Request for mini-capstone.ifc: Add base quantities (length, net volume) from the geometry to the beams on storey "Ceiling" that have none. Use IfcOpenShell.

First a look at what the model holds.

```python
import ifcopenshell
import ifcopenshell.util.element
import ifcopenshell.util.unit

model = ifcopenshell.open("mini-capstone.ifc")
print(model.schema)
for unit_type in ("LENGTHUNIT", "AREAUNIT", "VOLUMEUNIT"):
    print(unit_type, ifcopenshell.util.unit.calculate_unit_scale(model, unit_type))
storey = next(s for s in model.by_type("IfcBuildingStorey") if s.Name == "Ceiling")
beams = [e for e in ifcopenshell.util.element.get_decomposition(storey) if e.is_a("IfcBeam")]
for e in sorted(beams, key=lambda e: e.id()):
    print(e.id(), e.is_a(), e.Name, list(ifcopenshell.util.element.get_psets(e, qtos_only=True)), sep=" | ")
```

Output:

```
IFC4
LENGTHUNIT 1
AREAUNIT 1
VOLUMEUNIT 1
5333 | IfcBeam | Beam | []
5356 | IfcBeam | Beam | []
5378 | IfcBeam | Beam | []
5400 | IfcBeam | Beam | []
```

```python
import ifcopenshell
import ifcopenshell.api.pset
import ifcopenshell.geom
import ifcopenshell.util.element
import ifcopenshell.util.shape
import ifcopenshell.util.unit

model = ifcopenshell.open("mini-capstone.ifc")
unit_scale = ifcopenshell.util.unit.calculate_unit_scale(model)
volume_scale = ifcopenshell.util.unit.calculate_unit_scale(model, "VOLUMEUNIT")
settings = ifcopenshell.geom.settings()

storey = next(s for s in model.by_type("IfcBuildingStorey") if s.Name == "Ceiling")
beams = [e for e in ifcopenshell.util.element.get_decomposition(storey) if e.is_a("IfcBeam")]

for e in sorted(beams, key=lambda e: e.id()):
    if ifcopenshell.util.element.get_psets(e, qtos_only=True, should_inherit=False):
        continue
    # Geometry comes back in metres, in the element's own axes.
    shape = ifcopenshell.geom.create_shape(settings, e)
    values = {
        "Length": ifcopenshell.util.shape.get_max_xyz(shape.geometry) / unit_scale,
        "NetVolume": ifcopenshell.util.shape.get_volume(shape.geometry) / volume_scale,
    }
    qto = ifcopenshell.api.pset.add_qto(model, product=e, name="Qto_BeamBaseQuantities")
    ifcopenshell.api.pset.edit_qto(model, qto=qto, properties=values)
    print(e.id(), {k: round(v, 3) for k, v in values.items()})

model.write("mini-capstone_edited.ifc")
```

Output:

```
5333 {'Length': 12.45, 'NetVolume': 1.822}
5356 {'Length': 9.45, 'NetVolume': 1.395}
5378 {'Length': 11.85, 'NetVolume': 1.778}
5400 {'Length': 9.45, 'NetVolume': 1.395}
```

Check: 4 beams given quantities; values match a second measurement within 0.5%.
